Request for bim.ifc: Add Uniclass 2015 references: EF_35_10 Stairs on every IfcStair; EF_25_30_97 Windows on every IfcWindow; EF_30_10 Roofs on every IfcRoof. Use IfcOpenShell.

First a look at what the model holds.

```python
import ifcopenshell

model = ifcopenshell.open("bim.ifc")
print(model.schema)
print("classifications:", [c.Name for c in model.by_type("IfcClassification")])
for ifc_class in ("IfcDoor", "IfcRoof", "IfcStair", "IfcWall", "IfcWindow"):
    print(ifc_class, len(model.by_type(ifc_class)))
```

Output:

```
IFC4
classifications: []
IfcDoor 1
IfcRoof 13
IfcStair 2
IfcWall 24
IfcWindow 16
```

```python
import ifcopenshell
import ifcopenshell.api.classification

model = ifcopenshell.open("bim.ifc")

system = ifcopenshell.api.classification.add_classification(model, classification="Uniclass 2015")

codes = {
    "IfcStair": ("EF_35_10", "Stairs"),
    "IfcWindow": ("EF_25_30_97", "Windows"),
    "IfcRoof": ("EF_30_10", "Roofs"),
}
for ifc_class, (code, name) in codes.items():
    products = model.by_type(ifc_class)
    ifcopenshell.api.classification.add_reference(
        model, products=products, classification=system, identification=code, name=name
    )
    print(code, len(products))

model.write("bim_v2.ifc")
```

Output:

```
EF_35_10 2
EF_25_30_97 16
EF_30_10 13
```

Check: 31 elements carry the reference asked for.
